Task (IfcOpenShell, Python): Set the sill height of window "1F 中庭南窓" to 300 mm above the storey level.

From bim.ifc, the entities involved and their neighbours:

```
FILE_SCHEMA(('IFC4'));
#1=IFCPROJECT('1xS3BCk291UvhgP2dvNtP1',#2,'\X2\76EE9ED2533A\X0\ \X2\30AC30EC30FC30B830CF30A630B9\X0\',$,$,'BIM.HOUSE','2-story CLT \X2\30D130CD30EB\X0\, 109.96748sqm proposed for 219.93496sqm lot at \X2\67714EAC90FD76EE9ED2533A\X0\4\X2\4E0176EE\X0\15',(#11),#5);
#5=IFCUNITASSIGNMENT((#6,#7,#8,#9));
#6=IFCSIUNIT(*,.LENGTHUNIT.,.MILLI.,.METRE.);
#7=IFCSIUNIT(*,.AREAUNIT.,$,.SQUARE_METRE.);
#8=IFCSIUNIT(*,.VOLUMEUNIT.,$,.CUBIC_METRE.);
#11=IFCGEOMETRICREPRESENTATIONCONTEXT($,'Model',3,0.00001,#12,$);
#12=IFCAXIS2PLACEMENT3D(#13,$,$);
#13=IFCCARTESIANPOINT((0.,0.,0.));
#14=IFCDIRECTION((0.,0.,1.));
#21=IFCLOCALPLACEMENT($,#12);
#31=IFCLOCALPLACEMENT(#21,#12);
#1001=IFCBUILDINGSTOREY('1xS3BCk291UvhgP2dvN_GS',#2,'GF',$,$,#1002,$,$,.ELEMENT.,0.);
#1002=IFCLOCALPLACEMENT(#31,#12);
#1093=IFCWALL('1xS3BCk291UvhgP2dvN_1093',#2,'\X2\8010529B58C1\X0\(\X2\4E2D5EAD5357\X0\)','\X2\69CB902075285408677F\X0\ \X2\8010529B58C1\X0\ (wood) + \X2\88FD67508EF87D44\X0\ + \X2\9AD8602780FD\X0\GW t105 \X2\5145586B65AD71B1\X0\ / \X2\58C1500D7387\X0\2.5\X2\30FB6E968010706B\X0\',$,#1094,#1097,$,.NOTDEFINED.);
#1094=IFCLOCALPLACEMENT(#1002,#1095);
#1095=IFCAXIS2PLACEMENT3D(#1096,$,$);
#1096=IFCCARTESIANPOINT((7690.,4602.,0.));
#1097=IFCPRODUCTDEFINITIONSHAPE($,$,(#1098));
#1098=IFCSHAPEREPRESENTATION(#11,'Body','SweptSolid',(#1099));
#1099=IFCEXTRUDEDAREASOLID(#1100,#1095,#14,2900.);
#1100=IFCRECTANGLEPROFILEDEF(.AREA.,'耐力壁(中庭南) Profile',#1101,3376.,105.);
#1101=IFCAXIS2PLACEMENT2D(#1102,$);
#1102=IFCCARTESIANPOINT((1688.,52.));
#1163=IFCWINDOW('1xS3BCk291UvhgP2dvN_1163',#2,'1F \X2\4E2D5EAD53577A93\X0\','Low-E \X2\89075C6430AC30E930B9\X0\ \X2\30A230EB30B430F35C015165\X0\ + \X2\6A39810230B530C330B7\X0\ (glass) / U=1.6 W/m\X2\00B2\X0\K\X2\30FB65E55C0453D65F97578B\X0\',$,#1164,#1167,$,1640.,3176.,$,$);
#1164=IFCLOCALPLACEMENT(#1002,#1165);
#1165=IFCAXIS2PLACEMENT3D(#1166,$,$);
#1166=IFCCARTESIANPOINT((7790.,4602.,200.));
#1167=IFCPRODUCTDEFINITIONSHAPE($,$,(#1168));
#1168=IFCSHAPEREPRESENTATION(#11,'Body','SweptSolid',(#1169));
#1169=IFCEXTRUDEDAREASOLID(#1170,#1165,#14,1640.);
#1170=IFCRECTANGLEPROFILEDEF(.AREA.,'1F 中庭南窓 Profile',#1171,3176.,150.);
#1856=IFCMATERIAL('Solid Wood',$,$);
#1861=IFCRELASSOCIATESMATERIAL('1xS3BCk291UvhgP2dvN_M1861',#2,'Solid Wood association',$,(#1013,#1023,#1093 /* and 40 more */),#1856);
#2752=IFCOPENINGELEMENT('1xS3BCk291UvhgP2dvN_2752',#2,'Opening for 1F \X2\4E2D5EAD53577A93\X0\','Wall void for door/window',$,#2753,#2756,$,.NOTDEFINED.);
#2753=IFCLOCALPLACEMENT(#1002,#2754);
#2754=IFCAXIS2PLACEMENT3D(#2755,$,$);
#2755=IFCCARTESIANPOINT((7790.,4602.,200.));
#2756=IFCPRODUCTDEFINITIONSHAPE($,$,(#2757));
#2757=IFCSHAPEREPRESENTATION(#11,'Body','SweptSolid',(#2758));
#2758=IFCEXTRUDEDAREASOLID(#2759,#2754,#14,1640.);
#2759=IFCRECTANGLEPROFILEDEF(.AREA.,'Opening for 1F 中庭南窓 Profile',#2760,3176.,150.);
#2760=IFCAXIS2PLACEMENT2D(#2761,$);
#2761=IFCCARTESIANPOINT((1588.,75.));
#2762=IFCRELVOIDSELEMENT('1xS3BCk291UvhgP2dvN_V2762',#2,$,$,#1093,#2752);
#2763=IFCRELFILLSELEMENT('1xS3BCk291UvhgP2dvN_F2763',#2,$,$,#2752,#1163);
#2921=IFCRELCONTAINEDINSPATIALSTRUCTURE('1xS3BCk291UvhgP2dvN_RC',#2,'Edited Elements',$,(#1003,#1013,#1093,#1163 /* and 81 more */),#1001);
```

```python
import numpy as np
import ifcopenshell
import ifcopenshell.api.geometry
import ifcopenshell.geom
import ifcopenshell.util.element
import ifcopenshell.util.placement
import ifcopenshell.util.shape
import ifcopenshell.util.unit

model = ifcopenshell.open("bim.ifc")
unit_scale = ifcopenshell.util.unit.calculate_unit_scale(model)

window = model.by_guid("1xS3BCk291UvhgP2dvN_1163")
opening = window.FillsVoids[0].RelatingOpeningElement
storey = ifcopenshell.util.element.get_container(window, ifc_class="IfcBuildingStorey")
level = ifcopenshell.util.placement.get_local_placement(storey.ObjectPlacement)[2, 3]

# The opening's origin need not be at the sill, so measure its lowest point.
shape = ifcopenshell.geom.create_shape(ifcopenshell.geom.settings(), opening)
bottom = ifcopenshell.util.shape.get_shape_bottom_elevation(shape, shape.geometry) / unit_scale
dz = level + 0.3 / unit_scale - bottom

shift = np.array([0.0, 0.0, dz])
# The window is not placed relative to its opening, so move both.
for product in (opening, window):
    matrix = ifcopenshell.util.placement.get_local_placement(product.ObjectPlacement)
    matrix[:3, 3] += shift
    ifcopenshell.api.geometry.edit_object_placement(model, product=product, matrix=matrix, is_si=False)

print(f"moved by {dz * unit_scale:+.3f} m")

model.write("bim-out.ifc")
```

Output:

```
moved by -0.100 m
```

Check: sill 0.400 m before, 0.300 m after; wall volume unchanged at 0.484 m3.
